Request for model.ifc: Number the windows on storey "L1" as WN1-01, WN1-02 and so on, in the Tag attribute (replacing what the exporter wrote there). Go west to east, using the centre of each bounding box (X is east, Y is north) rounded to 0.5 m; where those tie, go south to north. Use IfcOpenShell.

First a look at what the model holds.

```python
import ifcopenshell
import ifcopenshell.util.element
import ifcopenshell.util.placement

model = ifcopenshell.open("model.ifc")
print(model.schema)
storey = next(s for s in model.by_type("IfcBuildingStorey") if s.Name == "L1")
windows = [e for e in ifcopenshell.util.element.get_decomposition(storey) if e.is_a("IfcWindow")]
for e in sorted(windows, key=lambda e: e.id()):
    origin = ifcopenshell.util.placement.get_local_placement(e.ObjectPlacement)[:3, 3]
    print(e.id(), e.Tag, e.Name, origin.round(2) + 0.0, sep=" | ")
```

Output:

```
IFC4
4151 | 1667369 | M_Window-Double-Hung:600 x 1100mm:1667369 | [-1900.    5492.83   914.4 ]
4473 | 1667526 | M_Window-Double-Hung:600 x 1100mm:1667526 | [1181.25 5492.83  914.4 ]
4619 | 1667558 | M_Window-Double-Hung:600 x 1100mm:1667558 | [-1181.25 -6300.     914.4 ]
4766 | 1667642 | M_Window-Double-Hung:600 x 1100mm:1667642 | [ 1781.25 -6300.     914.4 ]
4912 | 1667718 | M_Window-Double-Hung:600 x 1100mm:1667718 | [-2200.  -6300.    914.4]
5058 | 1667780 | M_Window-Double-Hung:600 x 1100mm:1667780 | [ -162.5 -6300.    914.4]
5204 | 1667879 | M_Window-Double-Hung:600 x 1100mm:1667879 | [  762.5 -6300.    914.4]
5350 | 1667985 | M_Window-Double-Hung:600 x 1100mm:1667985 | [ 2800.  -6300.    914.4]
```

```python
import ifcopenshell
import ifcopenshell.geom
import ifcopenshell.util.element
import ifcopenshell.util.shape

model = ifcopenshell.open("model.ifc")
settings = ifcopenshell.geom.settings()
settings.set("use-world-coords", True)


def centre(element):
    shape = ifcopenshell.geom.create_shape(settings, element)
    return ifcopenshell.util.shape.get_bbox_centroid(shape.geometry)


storey = next(s for s in model.by_type("IfcBuildingStorey") if s.Name == "L1")
windows = [e for e in ifcopenshell.util.element.get_decomposition(storey) if e.is_a("IfcWindow")]

# Insertion points can sit at a corner or the storey origin, so sort by the geometry (in metres).
centres = {e: centre(e) for e in windows}
windows.sort(key=lambda e: (round(centres[e][0] / 0.5), centres[e][1]))

for i, e in enumerate(windows, start=1):
    number = f"WN1-{i:02d}"
    e.Tag = number
    print(e.id(), number)

model.write("model-out.ifc")
```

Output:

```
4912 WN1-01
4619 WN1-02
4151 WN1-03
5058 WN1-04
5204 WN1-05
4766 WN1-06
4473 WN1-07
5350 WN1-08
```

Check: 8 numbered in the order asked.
